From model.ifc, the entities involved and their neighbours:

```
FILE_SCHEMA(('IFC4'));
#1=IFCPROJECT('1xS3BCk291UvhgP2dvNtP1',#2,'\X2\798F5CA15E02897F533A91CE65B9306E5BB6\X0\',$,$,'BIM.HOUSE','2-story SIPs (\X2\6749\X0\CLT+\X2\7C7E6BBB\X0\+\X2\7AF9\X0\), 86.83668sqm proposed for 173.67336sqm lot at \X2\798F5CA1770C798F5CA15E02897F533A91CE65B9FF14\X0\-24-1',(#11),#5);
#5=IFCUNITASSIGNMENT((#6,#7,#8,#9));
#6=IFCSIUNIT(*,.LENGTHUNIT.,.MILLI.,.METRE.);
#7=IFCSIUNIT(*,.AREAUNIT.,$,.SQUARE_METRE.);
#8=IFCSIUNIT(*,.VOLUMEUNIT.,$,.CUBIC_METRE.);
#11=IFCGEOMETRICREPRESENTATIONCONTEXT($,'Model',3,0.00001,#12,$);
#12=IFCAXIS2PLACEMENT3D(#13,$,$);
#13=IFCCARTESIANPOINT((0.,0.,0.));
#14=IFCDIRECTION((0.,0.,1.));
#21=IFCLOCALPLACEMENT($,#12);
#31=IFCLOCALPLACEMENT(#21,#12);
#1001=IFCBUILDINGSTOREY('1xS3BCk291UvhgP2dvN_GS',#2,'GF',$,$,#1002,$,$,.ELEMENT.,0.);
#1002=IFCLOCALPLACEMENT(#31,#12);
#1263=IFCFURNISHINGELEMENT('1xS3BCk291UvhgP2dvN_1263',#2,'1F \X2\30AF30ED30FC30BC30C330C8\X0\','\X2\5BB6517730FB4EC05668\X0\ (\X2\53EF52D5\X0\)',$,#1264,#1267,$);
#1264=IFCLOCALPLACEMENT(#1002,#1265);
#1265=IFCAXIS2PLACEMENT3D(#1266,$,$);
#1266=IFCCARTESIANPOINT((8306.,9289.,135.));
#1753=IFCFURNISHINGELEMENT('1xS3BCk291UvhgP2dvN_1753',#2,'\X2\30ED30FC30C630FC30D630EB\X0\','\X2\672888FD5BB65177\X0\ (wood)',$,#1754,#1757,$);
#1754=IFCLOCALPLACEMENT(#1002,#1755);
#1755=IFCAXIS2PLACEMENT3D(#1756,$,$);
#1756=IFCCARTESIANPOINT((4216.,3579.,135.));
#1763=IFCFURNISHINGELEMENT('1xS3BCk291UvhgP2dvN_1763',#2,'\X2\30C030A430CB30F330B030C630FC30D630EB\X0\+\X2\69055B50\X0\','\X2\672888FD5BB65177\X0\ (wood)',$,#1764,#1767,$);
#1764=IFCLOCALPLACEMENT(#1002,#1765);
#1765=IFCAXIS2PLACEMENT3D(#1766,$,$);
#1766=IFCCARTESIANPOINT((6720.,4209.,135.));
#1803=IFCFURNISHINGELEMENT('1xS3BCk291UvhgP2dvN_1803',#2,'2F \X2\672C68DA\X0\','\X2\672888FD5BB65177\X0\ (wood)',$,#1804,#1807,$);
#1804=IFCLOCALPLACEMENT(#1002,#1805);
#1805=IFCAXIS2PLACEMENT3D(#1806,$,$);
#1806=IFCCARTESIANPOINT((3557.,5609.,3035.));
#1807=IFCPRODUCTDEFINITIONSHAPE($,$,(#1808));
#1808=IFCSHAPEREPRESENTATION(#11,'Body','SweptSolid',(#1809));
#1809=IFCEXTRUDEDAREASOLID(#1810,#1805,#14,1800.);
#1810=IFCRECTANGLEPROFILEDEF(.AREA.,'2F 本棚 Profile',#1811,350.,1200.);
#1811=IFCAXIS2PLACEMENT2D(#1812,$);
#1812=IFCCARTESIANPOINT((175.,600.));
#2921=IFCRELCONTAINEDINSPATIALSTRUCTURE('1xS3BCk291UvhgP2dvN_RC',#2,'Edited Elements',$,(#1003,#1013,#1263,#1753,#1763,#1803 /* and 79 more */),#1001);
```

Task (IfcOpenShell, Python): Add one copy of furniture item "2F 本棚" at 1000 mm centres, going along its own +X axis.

```python
import ifcopenshell
import ifcopenshell.api.geometry
import ifcopenshell.api.root
import ifcopenshell.util.element
import ifcopenshell.util.placement

model = ifcopenshell.open("model.ifc")


def reuse_history(source, copy):
    """copy_class also copies each property set's owner history, people and application; keep the originals."""
    for rel in copy.IsDefinedBy:
        if rel.is_a("IfcRelDefinesByProperties") and (history := rel.RelatingPropertyDefinition.OwnerHistory):
            rel.RelatingPropertyDefinition.OwnerHistory = source.OwnerHistory
            ifcopenshell.util.element.remove_deep2(model, history)


source = model.by_guid("1xS3BCk291UvhgP2dvN_1803")
base = ifcopenshell.util.placement.get_local_placement(source.ObjectPlacement)
step = base[:3, 0] * 1000.0

for i in range(1, 2):
    copy = ifcopenshell.api.root.copy_class(model, product=source)
    copy.Representation = ifcopenshell.util.element.copy_deep(
        model, source.Representation, exclude=["IfcGeometricRepresentationContext", "IfcRepresentationMap"]
    )
    reuse_history(source, copy)
    matrix = base.copy()
    matrix[:3, 3] += i * step
    print("added at", matrix[:3, 3].round(3) + 0.0)
    ifcopenshell.api.geometry.edit_object_placement(model, product=copy, matrix=matrix, is_si=False)

model.write("model_edited.ifc")
```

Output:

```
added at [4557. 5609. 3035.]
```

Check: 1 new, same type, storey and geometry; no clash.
